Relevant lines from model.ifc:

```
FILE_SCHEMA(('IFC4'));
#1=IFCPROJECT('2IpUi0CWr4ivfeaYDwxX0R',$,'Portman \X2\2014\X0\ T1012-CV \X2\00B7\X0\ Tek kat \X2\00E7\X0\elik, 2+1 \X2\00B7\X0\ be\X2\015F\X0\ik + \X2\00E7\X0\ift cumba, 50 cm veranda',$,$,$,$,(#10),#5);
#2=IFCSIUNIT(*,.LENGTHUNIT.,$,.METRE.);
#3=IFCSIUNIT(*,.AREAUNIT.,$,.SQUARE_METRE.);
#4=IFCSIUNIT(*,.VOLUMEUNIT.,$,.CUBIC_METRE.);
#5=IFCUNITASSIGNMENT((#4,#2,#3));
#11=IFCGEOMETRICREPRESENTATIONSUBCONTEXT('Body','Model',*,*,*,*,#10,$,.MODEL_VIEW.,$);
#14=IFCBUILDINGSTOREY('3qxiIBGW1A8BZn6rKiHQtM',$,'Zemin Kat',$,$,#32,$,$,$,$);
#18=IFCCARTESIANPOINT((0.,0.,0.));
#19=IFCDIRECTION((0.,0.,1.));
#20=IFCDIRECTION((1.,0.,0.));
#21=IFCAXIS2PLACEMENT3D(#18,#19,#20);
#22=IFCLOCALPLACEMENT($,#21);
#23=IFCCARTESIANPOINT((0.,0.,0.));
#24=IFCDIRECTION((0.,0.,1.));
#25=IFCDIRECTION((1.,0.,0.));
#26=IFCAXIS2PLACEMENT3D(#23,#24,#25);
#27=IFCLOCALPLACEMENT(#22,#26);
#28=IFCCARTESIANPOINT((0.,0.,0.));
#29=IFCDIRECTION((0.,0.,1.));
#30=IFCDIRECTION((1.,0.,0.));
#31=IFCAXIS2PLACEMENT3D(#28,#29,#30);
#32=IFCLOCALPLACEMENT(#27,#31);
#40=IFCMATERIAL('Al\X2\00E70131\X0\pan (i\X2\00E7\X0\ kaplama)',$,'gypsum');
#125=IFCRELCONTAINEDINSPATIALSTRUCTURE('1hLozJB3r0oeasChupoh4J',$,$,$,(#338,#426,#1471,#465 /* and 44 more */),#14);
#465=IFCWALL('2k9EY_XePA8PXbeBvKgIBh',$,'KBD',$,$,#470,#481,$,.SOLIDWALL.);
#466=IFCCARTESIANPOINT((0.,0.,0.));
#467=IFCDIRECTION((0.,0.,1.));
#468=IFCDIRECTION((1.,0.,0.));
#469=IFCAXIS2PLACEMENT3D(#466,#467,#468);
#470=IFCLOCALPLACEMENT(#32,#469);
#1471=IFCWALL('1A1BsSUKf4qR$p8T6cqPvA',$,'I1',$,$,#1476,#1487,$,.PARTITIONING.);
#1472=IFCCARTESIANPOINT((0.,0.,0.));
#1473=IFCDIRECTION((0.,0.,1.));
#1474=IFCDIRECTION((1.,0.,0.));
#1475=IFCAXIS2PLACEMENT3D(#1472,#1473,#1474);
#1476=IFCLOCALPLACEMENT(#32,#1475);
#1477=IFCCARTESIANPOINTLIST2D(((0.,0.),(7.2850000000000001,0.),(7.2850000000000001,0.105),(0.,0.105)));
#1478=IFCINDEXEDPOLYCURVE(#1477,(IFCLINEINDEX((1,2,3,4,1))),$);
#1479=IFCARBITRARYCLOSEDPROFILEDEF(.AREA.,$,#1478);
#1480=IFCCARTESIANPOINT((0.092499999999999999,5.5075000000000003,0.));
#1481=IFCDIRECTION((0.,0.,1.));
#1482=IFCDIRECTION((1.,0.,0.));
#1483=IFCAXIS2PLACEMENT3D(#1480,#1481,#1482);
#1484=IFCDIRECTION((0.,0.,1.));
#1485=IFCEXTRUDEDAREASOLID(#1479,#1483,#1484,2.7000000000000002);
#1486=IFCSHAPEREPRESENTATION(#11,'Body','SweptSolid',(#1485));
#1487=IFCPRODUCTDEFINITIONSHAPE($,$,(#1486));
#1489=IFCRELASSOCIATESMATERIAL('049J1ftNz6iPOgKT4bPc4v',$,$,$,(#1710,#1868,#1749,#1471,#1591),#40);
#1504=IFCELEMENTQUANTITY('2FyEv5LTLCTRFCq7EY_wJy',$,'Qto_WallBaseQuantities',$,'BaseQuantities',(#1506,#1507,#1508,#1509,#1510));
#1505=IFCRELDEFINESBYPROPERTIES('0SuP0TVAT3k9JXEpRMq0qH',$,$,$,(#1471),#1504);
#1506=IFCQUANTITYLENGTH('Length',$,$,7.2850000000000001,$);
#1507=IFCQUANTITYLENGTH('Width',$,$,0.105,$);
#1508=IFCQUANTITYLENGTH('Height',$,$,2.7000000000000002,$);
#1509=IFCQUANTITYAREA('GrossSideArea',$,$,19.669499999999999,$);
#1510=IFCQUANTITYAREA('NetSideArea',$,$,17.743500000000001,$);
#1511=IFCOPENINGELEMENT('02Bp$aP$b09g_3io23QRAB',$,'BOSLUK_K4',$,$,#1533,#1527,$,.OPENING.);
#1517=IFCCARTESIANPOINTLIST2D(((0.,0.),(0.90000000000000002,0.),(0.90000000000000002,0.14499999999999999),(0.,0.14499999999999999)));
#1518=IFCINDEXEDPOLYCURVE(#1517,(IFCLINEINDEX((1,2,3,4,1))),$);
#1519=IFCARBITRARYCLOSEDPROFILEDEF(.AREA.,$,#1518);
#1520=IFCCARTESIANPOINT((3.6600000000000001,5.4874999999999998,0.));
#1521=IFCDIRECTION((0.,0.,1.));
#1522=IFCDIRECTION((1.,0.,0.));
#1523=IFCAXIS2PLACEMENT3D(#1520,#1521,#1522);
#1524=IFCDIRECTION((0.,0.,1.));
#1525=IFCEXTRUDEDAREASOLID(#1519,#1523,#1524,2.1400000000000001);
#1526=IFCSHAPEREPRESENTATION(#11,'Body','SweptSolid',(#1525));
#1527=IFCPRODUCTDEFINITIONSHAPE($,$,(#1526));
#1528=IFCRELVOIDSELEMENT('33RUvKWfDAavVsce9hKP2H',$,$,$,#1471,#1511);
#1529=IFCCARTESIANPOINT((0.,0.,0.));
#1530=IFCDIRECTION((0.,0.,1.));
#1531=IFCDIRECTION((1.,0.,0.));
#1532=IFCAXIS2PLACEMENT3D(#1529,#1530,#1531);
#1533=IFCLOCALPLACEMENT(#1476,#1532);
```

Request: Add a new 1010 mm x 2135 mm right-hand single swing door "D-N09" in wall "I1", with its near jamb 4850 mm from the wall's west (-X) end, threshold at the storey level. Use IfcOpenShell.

```python
import numpy as np
import ifcopenshell
import ifcopenshell.api.feature
import ifcopenshell.api.geometry
import ifcopenshell.api.pset
import ifcopenshell.api.root
import ifcopenshell.api.spatial
import ifcopenshell.geom
import ifcopenshell.util.element
import ifcopenshell.util.placement
import ifcopenshell.util.representation
import ifcopenshell.util.shape
import ifcopenshell.util.unit

model = ifcopenshell.open("model.ifc")
unit_scale = ifcopenshell.util.unit.calculate_unit_scale(model)
area_scale = ifcopenshell.util.unit.calculate_unit_scale(model, "AREAUNIT")
settings = ifcopenshell.geom.settings()


def volume(element):
    """Net volume in cubic metres, openings subtracted."""
    shape = ifcopenshell.geom.create_shape(settings, element)
    return ifcopenshell.util.shape.get_volume(shape.geometry)


wall = model.by_guid("1A1BsSUKf4qR$p8T6cqPvA")
storey = ifcopenshell.util.element.get_container(wall, ifc_class="IfcBuildingStorey")
context = ifcopenshell.util.representation.get_context(model, "Model", "Body", "MODEL_VIEW")
before = volume(wall)

width, height, from_end, sill = 1.01, 2.135, 4.85, 0.0  # metres

# The wall runs along its own X axis, and the end named is its -X end.
wall_shape = ifcopenshell.geom.create_shape(settings, wall)
x, y, z = ifcopenshell.util.shape.get_vertices(wall_shape.geometry).T
start = x.min() + from_end
face, thickness = float(y.min()), float(y.max() - y.min())
wall_matrix = ifcopenshell.util.placement.get_local_placement(wall.ObjectPlacement)
level = ifcopenshell.util.placement.get_local_placement(storey.ObjectPlacement)[2, 3]


def in_wall(x, y):
    """Placement at x, y metres in the wall's axes, at sill height."""
    matrix = wall_matrix.copy()
    matrix[:, 3] = wall_matrix @ np.array([x / unit_scale, y / unit_scale, 0.0, 1.0])
    matrix[2, 3] = level + sill / unit_scale
    return matrix


# Opening: a box that overshoots both wall faces by 50 mm.
opening = ifcopenshell.api.root.create_entity(model, ifc_class="IfcOpeningElement", predefined_type="OPENING")
box = ifcopenshell.api.geometry.add_wall_representation(
    model, context=context, length=width, height=height, thickness=thickness + 0.1
)
ifcopenshell.api.geometry.assign_representation(model, product=opening, representation=box)
ifcopenshell.api.geometry.edit_object_placement(model, product=opening, matrix=in_wall(start, face - 0.05), is_si=False)
ifcopenshell.api.feature.add_feature(model, feature=opening, element=wall)

door = ifcopenshell.api.root.create_entity(model, ifc_class="IfcDoor", name="D-N09", predefined_type="DOOR")
door.OverallWidth, door.OverallHeight = width / unit_scale, height / unit_scale
door.OperationType = "SINGLE_SWING_RIGHT"
body = ifcopenshell.api.geometry.add_door_representation(
    model,
    context=context,
    overall_width=door.OverallWidth,
    overall_height=door.OverallHeight,
    operation_type="SINGLE_SWING_RIGHT",
    lining_properties={"LiningDepth": thickness / unit_scale, "ThresholdDepth": thickness / unit_scale},
)
ifcopenshell.api.geometry.assign_representation(model, product=door, representation=body)
ifcopenshell.api.spatial.assign_container(model, products=[door], relating_structure=storey)
ifcopenshell.api.feature.add_filling(model, opening=opening, element=door)

# The lining spans the wall, so the door starts at the wall face.
ifcopenshell.api.geometry.edit_object_placement(model, product=door, matrix=in_wall(start, face), is_si=False)

after = volume(wall)

# Update the wall's stored quantities.
qto = model.by_id(ifcopenshell.util.element.get_pset(wall, "Qto_WallBaseQuantities", should_inherit=False)["id"])
ifcopenshell.api.pset.edit_qto(model, qto=qto, properties={"NetSideArea": after / thickness / area_scale})

print(f"wall volume {before:.3f} -> {after:.3f} m3")

model.write("model_v2.ifc")
```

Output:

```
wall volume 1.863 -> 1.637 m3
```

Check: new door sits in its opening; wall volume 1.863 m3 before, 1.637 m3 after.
